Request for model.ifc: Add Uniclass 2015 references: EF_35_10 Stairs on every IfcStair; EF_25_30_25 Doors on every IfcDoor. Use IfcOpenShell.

First a look at what the model holds.

```python
import ifcopenshell

model = ifcopenshell.open("model.ifc")
print(model.schema)
print("classifications:", [c.Name for c in model.by_type("IfcClassification")])
for ifc_class in ("IfcDoor", "IfcRoof", "IfcStair", "IfcWall", "IfcWindow"):
    print(ifc_class, len(model.by_type(ifc_class)))
```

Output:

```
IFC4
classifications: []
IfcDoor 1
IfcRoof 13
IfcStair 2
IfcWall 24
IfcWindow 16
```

```python
import ifcopenshell
import ifcopenshell.api.classification

model = ifcopenshell.open("model.ifc")

system = ifcopenshell.api.classification.add_classification(model, classification="Uniclass 2015")

codes = {
    "IfcStair": ("EF_35_10", "Stairs"),
    "IfcDoor": ("EF_25_30_25", "Doors"),
}
for ifc_class, (code, name) in codes.items():
    products = model.by_type(ifc_class)
    ifcopenshell.api.classification.add_reference(
        model, products=products, classification=system, identification=code, name=name
    )
    print(code, len(products))

model.write("model_updated.ifc")
```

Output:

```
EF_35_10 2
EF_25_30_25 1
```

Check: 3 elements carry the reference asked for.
